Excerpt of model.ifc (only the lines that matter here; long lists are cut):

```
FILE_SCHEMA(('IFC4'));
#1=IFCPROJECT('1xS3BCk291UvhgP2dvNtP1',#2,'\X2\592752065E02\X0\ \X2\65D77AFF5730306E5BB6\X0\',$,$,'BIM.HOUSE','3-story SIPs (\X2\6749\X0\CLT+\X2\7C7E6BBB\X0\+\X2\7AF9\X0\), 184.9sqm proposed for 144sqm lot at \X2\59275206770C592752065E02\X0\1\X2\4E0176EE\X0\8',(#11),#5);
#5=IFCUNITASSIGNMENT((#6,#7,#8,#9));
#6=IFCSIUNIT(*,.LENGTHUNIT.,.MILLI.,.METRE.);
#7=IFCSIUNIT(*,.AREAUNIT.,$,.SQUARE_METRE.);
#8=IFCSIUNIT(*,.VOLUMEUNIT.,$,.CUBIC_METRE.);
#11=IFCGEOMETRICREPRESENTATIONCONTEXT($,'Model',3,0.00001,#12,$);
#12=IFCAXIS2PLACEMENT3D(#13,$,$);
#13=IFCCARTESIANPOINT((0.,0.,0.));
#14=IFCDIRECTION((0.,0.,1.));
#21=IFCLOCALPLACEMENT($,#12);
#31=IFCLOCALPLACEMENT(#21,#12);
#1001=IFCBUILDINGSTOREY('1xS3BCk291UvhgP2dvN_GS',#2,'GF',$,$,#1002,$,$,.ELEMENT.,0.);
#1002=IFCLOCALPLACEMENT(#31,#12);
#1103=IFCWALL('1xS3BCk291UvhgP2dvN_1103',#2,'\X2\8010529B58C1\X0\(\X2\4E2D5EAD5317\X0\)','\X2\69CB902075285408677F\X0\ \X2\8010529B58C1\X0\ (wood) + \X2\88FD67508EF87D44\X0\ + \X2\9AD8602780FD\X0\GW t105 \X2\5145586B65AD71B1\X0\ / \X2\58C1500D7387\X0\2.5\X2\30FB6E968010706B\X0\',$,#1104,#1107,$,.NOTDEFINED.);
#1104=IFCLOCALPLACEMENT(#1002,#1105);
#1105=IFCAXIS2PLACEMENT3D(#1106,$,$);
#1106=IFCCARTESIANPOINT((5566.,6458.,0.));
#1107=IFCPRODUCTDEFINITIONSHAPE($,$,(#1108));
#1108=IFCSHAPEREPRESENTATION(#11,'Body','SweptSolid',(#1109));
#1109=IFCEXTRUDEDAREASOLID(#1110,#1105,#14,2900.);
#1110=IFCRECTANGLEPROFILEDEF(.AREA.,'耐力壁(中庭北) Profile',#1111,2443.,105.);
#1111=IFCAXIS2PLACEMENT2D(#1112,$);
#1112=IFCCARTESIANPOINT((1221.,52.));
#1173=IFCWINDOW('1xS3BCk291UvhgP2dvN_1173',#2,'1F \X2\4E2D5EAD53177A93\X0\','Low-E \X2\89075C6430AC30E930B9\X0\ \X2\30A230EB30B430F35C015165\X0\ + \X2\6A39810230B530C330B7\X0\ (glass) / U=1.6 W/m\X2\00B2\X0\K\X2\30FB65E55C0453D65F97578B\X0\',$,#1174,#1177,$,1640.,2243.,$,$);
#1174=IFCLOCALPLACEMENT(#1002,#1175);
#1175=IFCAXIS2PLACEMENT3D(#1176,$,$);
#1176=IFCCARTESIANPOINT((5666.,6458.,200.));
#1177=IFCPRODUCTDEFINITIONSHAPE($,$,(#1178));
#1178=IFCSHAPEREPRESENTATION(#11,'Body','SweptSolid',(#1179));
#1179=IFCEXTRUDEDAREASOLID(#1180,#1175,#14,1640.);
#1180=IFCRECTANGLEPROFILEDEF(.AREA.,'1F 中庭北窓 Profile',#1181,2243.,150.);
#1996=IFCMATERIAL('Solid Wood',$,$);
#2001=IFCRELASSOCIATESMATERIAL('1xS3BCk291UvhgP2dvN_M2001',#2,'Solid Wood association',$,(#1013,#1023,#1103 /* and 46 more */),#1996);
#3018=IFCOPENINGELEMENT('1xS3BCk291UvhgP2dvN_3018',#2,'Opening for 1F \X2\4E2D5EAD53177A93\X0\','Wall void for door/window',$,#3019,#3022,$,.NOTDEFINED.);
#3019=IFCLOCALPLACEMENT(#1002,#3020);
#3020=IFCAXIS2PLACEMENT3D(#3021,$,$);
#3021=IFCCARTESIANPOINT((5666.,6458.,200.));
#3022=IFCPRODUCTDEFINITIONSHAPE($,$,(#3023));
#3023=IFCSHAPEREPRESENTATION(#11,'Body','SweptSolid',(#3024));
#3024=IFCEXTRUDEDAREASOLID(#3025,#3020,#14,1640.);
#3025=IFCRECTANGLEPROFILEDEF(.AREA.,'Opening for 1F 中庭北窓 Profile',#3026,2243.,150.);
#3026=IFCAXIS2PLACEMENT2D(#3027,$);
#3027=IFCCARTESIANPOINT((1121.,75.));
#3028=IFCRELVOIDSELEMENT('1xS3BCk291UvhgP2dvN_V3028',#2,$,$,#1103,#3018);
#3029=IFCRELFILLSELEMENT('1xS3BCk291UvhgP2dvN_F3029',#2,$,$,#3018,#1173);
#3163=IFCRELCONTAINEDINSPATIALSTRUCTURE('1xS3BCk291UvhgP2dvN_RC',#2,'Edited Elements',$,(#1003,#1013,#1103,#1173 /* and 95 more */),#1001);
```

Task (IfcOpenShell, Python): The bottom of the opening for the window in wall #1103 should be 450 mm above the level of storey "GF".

```python
import numpy as np
import ifcopenshell
import ifcopenshell.api.geometry
import ifcopenshell.geom
import ifcopenshell.util.element
import ifcopenshell.util.placement
import ifcopenshell.util.shape
import ifcopenshell.util.unit

model = ifcopenshell.open("model.ifc")
unit_scale = ifcopenshell.util.unit.calculate_unit_scale(model)

window = model.by_guid("1xS3BCk291UvhgP2dvN_1173")
opening = window.FillsVoids[0].RelatingOpeningElement
storey = ifcopenshell.util.element.get_container(window, ifc_class="IfcBuildingStorey")
level = ifcopenshell.util.placement.get_local_placement(storey.ObjectPlacement)[2, 3]

# The opening's origin need not be at the sill, so measure its lowest point.
shape = ifcopenshell.geom.create_shape(ifcopenshell.geom.settings(), opening)
bottom = ifcopenshell.util.shape.get_shape_bottom_elevation(shape, shape.geometry) / unit_scale
dz = level + 0.45 / unit_scale - bottom

shift = np.array([0.0, 0.0, dz])
# The window is not placed relative to its opening, so move both.
for product in (opening, window):
    matrix = ifcopenshell.util.placement.get_local_placement(product.ObjectPlacement)
    matrix[:3, 3] += shift
    ifcopenshell.api.geometry.edit_object_placement(model, product=product, matrix=matrix, is_si=False)

print(f"moved by {dz * unit_scale:+.3f} m")

model.write("model-out.ifc")
```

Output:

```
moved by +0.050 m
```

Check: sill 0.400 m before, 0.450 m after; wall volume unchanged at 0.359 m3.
